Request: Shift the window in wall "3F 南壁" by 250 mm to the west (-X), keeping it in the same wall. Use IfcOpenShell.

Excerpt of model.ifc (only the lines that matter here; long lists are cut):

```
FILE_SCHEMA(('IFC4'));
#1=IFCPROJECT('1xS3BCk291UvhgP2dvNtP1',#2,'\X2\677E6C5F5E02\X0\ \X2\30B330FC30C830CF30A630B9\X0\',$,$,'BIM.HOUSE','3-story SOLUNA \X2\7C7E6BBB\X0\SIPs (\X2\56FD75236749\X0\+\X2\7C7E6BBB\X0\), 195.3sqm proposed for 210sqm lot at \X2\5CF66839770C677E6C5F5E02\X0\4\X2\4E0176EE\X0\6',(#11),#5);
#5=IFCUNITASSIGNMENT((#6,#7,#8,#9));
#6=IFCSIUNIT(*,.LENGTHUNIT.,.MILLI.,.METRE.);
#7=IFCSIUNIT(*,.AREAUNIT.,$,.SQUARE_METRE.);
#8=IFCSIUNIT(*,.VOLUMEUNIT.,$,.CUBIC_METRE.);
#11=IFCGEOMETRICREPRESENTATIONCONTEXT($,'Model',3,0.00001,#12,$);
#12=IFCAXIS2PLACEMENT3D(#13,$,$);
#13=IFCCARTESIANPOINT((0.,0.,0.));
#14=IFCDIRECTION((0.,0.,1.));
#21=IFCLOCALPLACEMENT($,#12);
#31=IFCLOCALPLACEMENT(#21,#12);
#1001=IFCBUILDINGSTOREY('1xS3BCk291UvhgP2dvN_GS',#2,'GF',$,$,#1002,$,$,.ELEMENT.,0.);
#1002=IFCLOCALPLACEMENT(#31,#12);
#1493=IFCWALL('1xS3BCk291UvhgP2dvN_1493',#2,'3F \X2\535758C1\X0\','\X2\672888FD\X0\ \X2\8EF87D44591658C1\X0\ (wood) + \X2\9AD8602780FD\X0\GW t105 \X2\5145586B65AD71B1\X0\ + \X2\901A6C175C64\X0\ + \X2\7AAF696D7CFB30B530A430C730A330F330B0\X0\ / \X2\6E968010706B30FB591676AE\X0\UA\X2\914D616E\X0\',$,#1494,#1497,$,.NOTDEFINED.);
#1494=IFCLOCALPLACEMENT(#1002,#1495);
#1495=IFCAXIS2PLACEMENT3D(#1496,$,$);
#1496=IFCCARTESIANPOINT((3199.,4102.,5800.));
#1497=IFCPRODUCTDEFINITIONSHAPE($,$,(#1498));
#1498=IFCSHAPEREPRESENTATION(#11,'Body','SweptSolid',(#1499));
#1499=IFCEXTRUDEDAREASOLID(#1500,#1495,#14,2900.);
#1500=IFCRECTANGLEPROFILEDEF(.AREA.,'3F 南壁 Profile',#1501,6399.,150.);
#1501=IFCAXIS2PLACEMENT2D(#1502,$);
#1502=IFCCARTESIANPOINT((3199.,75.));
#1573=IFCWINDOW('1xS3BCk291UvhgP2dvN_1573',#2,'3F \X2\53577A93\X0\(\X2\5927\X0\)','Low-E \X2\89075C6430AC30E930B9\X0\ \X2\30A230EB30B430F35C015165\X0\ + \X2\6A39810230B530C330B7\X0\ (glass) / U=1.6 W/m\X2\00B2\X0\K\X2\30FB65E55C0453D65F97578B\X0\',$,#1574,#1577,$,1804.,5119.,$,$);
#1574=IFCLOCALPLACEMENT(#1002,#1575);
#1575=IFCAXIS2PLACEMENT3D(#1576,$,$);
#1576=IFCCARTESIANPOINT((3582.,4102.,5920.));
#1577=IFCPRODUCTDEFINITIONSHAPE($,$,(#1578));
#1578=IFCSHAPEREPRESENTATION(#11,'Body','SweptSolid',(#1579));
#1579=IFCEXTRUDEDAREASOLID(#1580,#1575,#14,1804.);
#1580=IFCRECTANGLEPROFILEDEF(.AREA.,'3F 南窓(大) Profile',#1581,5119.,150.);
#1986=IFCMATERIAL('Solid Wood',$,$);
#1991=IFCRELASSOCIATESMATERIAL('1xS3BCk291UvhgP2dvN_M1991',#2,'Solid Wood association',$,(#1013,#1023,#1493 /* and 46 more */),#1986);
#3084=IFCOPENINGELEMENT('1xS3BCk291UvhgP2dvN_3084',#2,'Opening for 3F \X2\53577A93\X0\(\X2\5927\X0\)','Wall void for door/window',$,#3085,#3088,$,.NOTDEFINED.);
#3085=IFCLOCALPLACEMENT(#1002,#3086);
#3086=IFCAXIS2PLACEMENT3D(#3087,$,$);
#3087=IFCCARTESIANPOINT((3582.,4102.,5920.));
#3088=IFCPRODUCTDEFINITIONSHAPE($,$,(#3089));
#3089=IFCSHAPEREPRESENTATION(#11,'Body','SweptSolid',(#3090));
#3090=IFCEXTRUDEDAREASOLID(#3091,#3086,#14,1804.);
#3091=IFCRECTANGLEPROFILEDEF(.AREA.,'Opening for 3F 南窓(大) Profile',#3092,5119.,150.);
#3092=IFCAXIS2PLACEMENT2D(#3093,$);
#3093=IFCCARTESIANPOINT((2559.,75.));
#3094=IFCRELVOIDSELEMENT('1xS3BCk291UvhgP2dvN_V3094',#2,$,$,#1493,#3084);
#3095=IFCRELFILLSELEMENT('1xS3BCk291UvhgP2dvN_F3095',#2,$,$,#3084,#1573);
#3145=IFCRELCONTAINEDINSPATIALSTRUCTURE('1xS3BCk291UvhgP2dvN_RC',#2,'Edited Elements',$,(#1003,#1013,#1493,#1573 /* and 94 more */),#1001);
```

```python
import ifcopenshell
import ifcopenshell.api.geometry
import ifcopenshell.util.placement

model = ifcopenshell.open("model.ifc")

window = model.by_guid("1xS3BCk291UvhgP2dvN_1573")
opening = window.FillsVoids[0].RelatingOpeningElement
wall = opening.VoidsElements[0].RelatingBuildingElement

wall_matrix = ifcopenshell.util.placement.get_local_placement(wall.ObjectPlacement)
shift = wall_matrix[:3, 0] * -250.0
before = ifcopenshell.util.placement.get_local_placement(window.ObjectPlacement)[:3, 3].copy()

# The window is not placed relative to its opening, so move both.
for product in (opening, window):
    matrix = ifcopenshell.util.placement.get_local_placement(product.ObjectPlacement)
    matrix[:3, 3] += shift
    ifcopenshell.api.geometry.edit_object_placement(model, product=product, matrix=matrix, is_si=False)

after = ifcopenshell.util.placement.get_local_placement(window.ObjectPlacement)[:3, 3]
print("window moved by", (after - before).round(3) + 0.0)

model.write("model_v2.ifc")
```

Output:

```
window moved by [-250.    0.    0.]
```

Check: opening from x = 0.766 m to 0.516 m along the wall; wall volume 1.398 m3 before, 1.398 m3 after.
